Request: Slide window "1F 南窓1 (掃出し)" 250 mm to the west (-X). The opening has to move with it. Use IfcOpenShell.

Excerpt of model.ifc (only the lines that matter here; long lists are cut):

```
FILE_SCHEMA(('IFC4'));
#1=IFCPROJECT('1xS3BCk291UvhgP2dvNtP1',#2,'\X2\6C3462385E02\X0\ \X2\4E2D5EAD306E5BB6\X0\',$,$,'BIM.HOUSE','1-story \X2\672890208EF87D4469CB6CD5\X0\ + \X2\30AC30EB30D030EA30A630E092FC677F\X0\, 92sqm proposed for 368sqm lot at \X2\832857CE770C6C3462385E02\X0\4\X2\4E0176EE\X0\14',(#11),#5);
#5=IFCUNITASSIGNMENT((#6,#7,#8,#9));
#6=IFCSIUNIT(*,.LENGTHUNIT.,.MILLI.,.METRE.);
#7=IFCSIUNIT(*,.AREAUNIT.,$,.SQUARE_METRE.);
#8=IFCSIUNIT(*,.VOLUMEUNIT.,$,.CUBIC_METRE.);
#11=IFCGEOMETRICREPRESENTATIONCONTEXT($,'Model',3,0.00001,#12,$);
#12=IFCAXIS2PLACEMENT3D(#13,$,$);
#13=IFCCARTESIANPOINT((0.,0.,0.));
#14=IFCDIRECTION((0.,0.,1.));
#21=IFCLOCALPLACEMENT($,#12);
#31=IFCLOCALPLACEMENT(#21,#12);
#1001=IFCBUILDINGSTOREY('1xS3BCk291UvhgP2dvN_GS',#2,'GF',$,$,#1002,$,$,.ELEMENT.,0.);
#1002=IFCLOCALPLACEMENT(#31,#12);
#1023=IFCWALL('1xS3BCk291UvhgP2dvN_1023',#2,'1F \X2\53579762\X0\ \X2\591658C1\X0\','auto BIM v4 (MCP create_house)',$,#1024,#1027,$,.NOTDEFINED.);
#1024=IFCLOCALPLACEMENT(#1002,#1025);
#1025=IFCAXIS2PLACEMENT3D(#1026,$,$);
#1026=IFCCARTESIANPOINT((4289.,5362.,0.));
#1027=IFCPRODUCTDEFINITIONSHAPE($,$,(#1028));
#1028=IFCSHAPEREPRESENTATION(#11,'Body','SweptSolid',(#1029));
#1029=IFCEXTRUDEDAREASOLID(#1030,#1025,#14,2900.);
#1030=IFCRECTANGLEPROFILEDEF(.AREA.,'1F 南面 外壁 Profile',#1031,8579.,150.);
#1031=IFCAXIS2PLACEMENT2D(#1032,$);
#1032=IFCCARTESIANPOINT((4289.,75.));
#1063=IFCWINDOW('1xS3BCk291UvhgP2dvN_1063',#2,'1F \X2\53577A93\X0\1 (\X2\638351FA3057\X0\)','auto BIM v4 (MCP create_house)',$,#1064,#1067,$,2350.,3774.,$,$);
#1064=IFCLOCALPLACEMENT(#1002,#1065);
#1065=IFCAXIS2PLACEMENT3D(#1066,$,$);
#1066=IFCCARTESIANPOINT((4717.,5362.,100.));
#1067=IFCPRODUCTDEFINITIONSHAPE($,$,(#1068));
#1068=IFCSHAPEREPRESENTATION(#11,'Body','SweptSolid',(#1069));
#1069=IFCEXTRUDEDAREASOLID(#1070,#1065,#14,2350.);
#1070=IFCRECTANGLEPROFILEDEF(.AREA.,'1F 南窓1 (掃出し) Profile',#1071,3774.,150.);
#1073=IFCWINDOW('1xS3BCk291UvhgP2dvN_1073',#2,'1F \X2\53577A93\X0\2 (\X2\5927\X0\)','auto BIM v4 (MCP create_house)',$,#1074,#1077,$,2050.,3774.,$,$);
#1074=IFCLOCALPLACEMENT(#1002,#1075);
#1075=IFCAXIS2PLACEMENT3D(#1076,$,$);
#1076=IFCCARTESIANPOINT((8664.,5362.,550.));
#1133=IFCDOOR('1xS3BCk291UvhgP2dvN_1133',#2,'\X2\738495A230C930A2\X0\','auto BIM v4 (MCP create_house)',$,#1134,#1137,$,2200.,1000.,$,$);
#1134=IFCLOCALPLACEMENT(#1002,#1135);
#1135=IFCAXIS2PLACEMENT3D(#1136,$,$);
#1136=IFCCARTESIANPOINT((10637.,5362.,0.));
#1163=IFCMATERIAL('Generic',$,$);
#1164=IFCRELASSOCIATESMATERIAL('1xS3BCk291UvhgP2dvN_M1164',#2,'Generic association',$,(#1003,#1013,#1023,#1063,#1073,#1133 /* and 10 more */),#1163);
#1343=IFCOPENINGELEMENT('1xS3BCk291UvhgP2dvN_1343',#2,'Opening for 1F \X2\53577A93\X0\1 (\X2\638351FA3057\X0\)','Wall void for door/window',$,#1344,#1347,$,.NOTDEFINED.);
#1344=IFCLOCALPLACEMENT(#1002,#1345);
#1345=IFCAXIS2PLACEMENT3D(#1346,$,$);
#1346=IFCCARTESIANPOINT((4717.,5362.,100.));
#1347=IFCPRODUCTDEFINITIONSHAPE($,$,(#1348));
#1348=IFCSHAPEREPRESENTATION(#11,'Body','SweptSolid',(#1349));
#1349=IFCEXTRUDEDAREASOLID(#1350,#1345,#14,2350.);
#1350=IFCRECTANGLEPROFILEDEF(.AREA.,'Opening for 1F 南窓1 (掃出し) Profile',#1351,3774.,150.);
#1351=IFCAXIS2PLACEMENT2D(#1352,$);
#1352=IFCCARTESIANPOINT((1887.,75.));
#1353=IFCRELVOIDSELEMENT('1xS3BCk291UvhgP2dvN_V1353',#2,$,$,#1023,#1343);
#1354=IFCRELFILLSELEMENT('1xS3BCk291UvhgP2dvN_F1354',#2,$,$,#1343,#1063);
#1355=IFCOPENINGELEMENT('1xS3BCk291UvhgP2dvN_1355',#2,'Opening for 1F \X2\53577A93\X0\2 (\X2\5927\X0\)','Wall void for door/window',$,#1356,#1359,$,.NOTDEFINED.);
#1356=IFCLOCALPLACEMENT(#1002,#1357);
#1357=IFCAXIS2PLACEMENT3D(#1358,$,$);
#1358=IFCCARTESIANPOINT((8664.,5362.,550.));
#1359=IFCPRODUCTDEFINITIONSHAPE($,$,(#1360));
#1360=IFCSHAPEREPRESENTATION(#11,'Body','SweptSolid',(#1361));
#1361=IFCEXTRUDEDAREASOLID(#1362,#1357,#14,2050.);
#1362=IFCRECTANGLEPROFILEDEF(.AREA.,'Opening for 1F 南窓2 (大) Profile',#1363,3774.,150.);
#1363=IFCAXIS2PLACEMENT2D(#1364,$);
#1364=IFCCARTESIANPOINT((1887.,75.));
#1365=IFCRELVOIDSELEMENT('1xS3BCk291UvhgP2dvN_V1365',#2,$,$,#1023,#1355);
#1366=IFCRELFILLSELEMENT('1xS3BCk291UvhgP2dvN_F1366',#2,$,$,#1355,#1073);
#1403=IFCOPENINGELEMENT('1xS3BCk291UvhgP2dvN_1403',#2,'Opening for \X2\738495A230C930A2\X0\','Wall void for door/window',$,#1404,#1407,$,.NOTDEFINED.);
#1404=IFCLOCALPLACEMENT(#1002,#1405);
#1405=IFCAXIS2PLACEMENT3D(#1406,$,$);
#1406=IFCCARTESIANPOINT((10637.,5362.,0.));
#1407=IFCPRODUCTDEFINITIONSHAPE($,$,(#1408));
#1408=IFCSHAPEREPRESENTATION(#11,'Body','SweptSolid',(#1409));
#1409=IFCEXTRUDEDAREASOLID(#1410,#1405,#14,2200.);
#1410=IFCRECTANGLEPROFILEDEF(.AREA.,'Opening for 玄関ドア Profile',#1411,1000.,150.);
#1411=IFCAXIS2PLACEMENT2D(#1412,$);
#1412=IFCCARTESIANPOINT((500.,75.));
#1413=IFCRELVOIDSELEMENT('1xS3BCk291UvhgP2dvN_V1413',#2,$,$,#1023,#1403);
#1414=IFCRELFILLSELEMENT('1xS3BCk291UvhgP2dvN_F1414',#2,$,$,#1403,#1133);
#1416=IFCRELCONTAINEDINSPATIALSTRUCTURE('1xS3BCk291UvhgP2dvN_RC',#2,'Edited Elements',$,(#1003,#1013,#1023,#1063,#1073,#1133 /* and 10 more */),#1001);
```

```python
import ifcopenshell
import ifcopenshell.api.geometry
import ifcopenshell.util.placement

model = ifcopenshell.open("model.ifc")

window = model.by_guid("1xS3BCk291UvhgP2dvN_1063")
opening = window.FillsVoids[0].RelatingOpeningElement
wall = opening.VoidsElements[0].RelatingBuildingElement

wall_matrix = ifcopenshell.util.placement.get_local_placement(wall.ObjectPlacement)
shift = wall_matrix[:3, 0] * -250.0
before = ifcopenshell.util.placement.get_local_placement(window.ObjectPlacement)[:3, 3].copy()

# The window is not placed relative to its opening, so move both.
for product in (opening, window):
    matrix = ifcopenshell.util.placement.get_local_placement(product.ObjectPlacement)
    matrix[:3, 3] += shift
    ifcopenshell.api.geometry.edit_object_placement(model, product=product, matrix=matrix, is_si=False)

after = ifcopenshell.util.placement.get_local_placement(window.ObjectPlacement)[:3, 3]
print("window moved by", (after - before).round(3) + 0.0)

model.write("model-out.ifc")
```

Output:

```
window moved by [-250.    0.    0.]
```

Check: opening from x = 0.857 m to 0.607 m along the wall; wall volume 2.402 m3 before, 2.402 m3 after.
